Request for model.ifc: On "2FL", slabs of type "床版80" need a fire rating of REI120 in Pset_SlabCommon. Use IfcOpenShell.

First a look at what the model holds.

```python
import ifcopenshell
import ifcopenshell.util.element

model = ifcopenshell.open("model.ifc")
print(model.schema)
storey = next(s for s in model.by_type("IfcBuildingStorey") if s.Name == "2FL")
slabs = [e for e in ifcopenshell.util.element.get_decomposition(storey) if e.is_a("IfcSlab")]
seen = {}
for e in slabs:
    element_type = ifcopenshell.util.element.get_type(e)
    key = (element_type.Name if element_type != e and element_type else None, ifcopenshell.util.element.get_pset(e, "Pset_SlabCommon", "FireRating"))
    seen[key] = seen.get(key, 0) + 1
for (name, value), count in sorted(seen.items(), key=str):
    print(count, "x", name, "|", value)
```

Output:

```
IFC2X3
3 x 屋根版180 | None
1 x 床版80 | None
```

```python
import ifcopenshell
import ifcopenshell.api.pset
import ifcopenshell.util.element

model = ifcopenshell.open("model.ifc")

storey = next(s for s in model.by_type("IfcBuildingStorey") if s.Name == "2FL")
slabs = [e for e in ifcopenshell.util.element.get_decomposition(storey) if e.is_a("IfcSlab")]

count = 0
for e in slabs:
    element_type = ifcopenshell.util.element.get_type(e)
    if element_type in (None, e) or element_type.Name != "床版80":
        continue
    # add_pset returns the element's existing set when there is one.
    pset = ifcopenshell.api.pset.add_pset(model, product=e, name="Pset_SlabCommon")
    ifcopenshell.api.pset.edit_pset(model, pset=pset, properties={"FireRating": "REI120"})
    count += 1

print(count, "slabs updated")

model.write("model_v2.ifc")
```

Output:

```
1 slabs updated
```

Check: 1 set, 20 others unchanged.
